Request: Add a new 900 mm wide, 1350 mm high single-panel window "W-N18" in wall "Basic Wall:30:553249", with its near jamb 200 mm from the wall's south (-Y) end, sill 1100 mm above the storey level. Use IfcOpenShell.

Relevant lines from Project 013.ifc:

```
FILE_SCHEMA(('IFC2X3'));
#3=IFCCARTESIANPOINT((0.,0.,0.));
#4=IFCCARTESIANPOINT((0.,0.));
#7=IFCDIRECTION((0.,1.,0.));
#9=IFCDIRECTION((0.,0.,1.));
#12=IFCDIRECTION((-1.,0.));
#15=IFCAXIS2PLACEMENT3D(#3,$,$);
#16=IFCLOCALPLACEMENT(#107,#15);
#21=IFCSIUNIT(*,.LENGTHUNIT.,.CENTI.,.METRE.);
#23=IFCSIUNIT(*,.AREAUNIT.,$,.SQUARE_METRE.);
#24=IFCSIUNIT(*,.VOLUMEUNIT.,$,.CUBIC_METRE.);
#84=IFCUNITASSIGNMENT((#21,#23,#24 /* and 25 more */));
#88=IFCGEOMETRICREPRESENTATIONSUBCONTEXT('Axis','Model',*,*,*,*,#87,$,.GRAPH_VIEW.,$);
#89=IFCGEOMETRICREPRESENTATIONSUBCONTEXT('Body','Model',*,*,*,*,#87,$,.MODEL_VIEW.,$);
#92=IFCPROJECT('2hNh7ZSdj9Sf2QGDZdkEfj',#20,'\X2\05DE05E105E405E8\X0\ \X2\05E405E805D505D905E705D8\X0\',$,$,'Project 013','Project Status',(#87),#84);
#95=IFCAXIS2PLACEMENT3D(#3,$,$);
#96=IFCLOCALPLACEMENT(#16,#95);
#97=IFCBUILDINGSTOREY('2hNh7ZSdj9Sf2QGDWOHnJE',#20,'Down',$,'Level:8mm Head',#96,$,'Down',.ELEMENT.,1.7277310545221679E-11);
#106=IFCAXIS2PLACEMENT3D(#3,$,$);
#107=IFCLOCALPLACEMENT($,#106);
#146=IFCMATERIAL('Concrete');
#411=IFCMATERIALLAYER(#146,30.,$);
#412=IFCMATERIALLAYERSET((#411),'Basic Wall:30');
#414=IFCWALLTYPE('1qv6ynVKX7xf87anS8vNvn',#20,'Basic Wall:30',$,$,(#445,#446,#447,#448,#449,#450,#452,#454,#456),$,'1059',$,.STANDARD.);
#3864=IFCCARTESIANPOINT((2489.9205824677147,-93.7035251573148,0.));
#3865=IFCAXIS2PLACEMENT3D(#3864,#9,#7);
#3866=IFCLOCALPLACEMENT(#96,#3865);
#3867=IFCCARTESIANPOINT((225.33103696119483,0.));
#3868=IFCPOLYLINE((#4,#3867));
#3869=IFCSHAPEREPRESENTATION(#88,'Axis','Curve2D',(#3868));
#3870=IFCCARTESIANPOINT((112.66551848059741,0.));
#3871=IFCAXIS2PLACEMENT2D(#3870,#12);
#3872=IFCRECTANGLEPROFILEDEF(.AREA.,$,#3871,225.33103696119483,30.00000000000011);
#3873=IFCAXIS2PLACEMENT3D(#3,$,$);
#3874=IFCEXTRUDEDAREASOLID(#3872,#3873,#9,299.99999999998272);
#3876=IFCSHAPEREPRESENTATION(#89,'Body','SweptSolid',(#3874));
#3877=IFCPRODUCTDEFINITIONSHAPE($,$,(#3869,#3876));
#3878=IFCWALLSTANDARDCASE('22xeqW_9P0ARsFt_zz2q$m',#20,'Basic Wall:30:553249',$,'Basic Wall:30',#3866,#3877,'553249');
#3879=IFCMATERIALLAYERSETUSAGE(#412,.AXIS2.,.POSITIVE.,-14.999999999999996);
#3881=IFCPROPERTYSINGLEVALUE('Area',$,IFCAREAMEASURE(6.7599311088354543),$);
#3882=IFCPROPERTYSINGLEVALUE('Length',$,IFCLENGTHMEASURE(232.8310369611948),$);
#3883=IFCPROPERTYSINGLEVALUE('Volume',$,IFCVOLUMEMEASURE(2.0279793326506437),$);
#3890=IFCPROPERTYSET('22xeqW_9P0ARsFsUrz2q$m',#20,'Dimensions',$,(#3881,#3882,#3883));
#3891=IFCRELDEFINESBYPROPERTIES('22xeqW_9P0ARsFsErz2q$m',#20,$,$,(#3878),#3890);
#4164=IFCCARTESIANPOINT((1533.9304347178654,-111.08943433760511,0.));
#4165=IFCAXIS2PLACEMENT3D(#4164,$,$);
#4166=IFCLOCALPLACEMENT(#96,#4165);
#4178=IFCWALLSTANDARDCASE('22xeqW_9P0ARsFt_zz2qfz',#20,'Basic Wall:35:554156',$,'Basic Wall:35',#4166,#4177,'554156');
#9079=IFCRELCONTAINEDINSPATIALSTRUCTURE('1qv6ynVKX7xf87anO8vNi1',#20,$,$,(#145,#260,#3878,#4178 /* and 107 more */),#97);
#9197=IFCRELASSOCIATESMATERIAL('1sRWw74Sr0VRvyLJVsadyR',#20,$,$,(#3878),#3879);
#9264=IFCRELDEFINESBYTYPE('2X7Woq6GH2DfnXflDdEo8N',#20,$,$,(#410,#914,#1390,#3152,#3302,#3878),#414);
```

```python
import numpy as np
import ifcopenshell
import ifcopenshell.api.feature
import ifcopenshell.api.geometry
import ifcopenshell.api.pset
import ifcopenshell.api.root
import ifcopenshell.api.spatial
import ifcopenshell.api.type
import ifcopenshell.geom
import ifcopenshell.util.element
import ifcopenshell.util.placement
import ifcopenshell.util.representation
import ifcopenshell.util.shape
import ifcopenshell.util.unit

model = ifcopenshell.open("Project 013.ifc")
unit_scale = ifcopenshell.util.unit.calculate_unit_scale(model)
area_scale = ifcopenshell.util.unit.calculate_unit_scale(model, "AREAUNIT")
volume_scale = ifcopenshell.util.unit.calculate_unit_scale(model, "VOLUMEUNIT")
settings = ifcopenshell.geom.settings()


def volume(element):
    """Net volume in cubic metres, openings subtracted."""
    shape = ifcopenshell.geom.create_shape(settings, element)
    return ifcopenshell.util.shape.get_volume(shape.geometry)


wall = model.by_guid("22xeqW_9P0ARsFt_zz2q$m")
storey = ifcopenshell.util.element.get_container(wall, ifc_class="IfcBuildingStorey")
context = ifcopenshell.util.representation.get_context(model, "Model", "Body", "MODEL_VIEW")
before = volume(wall)

width, height, from_end, sill = 0.9, 1.35, 0.2, 1.1  # metres

# The wall runs along its own X axis, and the end named is its -X end.
wall_shape = ifcopenshell.geom.create_shape(settings, wall)
x, y, z = ifcopenshell.util.shape.get_vertices(wall_shape.geometry).T
start = x.min() + from_end
face, thickness = float(y.min()), float(y.max() - y.min())
wall_matrix = ifcopenshell.util.placement.get_local_placement(wall.ObjectPlacement)
level = ifcopenshell.util.placement.get_local_placement(storey.ObjectPlacement)[2, 3]


def in_wall(x, y):
    """Placement at x, y metres in the wall's axes, at sill height."""
    matrix = wall_matrix.copy()
    matrix[:, 3] = wall_matrix @ np.array([x / unit_scale, y / unit_scale, 0.0, 1.0])
    matrix[2, 3] = level + sill / unit_scale
    return matrix


# Opening: a box that overshoots both wall faces by 50 mm.
opening = ifcopenshell.api.root.create_entity(model, ifc_class="IfcOpeningElement")
box = ifcopenshell.api.geometry.add_wall_representation(
    model, context=context, length=width, height=height, thickness=thickness + 0.1
)
ifcopenshell.api.geometry.assign_representation(model, product=opening, representation=box)
ifcopenshell.api.geometry.edit_object_placement(model, product=opening, matrix=in_wall(start, face - 0.05), is_si=False)
ifcopenshell.api.feature.add_feature(model, feature=opening, element=wall)

window = ifcopenshell.api.root.create_entity(model, ifc_class="IfcWindow", name="W-N18")
window.OverallWidth, window.OverallHeight = width / unit_scale, height / unit_scale
body = ifcopenshell.api.geometry.add_window_representation(
    model,
    context=context,
    overall_width=window.OverallWidth,
    overall_height=window.OverallHeight,
    partition_type="SINGLE_PANEL",
)
ifcopenshell.api.geometry.assign_representation(model, product=window, representation=body)
ifcopenshell.api.spatial.assign_container(model, products=[window], relating_structure=storey)
fills = ifcopenshell.api.feature.add_filling(model, opening=opening, element=window)
fills.OwnerHistory = window.OwnerHistory  # required in IFC2X3

# IFC2X3 keeps the operation on the window style.
style = ifcopenshell.api.root.create_entity(model, ifc_class="IfcWindowStyle", name="W-N18")
style.OperationType, style.ConstructionType = "SINGLE_PANEL", "NOTDEFINED"
style.ParameterTakesPrecedence = style.Sizeable = False
ifcopenshell.api.type.assign_type(model, related_objects=[window], relating_type=style)

# Centre the window in the wall's thickness.
ifcopenshell.api.geometry.edit_object_placement(model, product=window, matrix=in_wall(start, face), is_si=False)
window_shape = ifcopenshell.geom.create_shape(settings, window)
depth = ifcopenshell.util.shape.get_vertices(window_shape.geometry)[:, 1]
offset = face + thickness / 2 - (depth.min() + depth.max()) / 2
ifcopenshell.api.geometry.edit_object_placement(model, product=window, matrix=in_wall(start, offset), is_si=False)

after = volume(wall)

# Update the wall's stored quantities.
pset = model.by_id(ifcopenshell.util.element.get_pset(wall, "Dimensions", should_inherit=False)["id"])
ifcopenshell.api.pset.edit_pset(model, pset=pset, properties={
    "Area": model.create_entity("IfcAreaMeasure", after / thickness / area_scale),
    "Volume": model.create_entity("IfcVolumeMeasure", after / volume_scale),
})

print(f"wall volume {before:.3f} -> {after:.3f} m3")

model.write("Project 013_edited.ifc")
```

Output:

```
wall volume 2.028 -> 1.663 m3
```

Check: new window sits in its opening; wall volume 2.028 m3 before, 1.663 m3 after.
